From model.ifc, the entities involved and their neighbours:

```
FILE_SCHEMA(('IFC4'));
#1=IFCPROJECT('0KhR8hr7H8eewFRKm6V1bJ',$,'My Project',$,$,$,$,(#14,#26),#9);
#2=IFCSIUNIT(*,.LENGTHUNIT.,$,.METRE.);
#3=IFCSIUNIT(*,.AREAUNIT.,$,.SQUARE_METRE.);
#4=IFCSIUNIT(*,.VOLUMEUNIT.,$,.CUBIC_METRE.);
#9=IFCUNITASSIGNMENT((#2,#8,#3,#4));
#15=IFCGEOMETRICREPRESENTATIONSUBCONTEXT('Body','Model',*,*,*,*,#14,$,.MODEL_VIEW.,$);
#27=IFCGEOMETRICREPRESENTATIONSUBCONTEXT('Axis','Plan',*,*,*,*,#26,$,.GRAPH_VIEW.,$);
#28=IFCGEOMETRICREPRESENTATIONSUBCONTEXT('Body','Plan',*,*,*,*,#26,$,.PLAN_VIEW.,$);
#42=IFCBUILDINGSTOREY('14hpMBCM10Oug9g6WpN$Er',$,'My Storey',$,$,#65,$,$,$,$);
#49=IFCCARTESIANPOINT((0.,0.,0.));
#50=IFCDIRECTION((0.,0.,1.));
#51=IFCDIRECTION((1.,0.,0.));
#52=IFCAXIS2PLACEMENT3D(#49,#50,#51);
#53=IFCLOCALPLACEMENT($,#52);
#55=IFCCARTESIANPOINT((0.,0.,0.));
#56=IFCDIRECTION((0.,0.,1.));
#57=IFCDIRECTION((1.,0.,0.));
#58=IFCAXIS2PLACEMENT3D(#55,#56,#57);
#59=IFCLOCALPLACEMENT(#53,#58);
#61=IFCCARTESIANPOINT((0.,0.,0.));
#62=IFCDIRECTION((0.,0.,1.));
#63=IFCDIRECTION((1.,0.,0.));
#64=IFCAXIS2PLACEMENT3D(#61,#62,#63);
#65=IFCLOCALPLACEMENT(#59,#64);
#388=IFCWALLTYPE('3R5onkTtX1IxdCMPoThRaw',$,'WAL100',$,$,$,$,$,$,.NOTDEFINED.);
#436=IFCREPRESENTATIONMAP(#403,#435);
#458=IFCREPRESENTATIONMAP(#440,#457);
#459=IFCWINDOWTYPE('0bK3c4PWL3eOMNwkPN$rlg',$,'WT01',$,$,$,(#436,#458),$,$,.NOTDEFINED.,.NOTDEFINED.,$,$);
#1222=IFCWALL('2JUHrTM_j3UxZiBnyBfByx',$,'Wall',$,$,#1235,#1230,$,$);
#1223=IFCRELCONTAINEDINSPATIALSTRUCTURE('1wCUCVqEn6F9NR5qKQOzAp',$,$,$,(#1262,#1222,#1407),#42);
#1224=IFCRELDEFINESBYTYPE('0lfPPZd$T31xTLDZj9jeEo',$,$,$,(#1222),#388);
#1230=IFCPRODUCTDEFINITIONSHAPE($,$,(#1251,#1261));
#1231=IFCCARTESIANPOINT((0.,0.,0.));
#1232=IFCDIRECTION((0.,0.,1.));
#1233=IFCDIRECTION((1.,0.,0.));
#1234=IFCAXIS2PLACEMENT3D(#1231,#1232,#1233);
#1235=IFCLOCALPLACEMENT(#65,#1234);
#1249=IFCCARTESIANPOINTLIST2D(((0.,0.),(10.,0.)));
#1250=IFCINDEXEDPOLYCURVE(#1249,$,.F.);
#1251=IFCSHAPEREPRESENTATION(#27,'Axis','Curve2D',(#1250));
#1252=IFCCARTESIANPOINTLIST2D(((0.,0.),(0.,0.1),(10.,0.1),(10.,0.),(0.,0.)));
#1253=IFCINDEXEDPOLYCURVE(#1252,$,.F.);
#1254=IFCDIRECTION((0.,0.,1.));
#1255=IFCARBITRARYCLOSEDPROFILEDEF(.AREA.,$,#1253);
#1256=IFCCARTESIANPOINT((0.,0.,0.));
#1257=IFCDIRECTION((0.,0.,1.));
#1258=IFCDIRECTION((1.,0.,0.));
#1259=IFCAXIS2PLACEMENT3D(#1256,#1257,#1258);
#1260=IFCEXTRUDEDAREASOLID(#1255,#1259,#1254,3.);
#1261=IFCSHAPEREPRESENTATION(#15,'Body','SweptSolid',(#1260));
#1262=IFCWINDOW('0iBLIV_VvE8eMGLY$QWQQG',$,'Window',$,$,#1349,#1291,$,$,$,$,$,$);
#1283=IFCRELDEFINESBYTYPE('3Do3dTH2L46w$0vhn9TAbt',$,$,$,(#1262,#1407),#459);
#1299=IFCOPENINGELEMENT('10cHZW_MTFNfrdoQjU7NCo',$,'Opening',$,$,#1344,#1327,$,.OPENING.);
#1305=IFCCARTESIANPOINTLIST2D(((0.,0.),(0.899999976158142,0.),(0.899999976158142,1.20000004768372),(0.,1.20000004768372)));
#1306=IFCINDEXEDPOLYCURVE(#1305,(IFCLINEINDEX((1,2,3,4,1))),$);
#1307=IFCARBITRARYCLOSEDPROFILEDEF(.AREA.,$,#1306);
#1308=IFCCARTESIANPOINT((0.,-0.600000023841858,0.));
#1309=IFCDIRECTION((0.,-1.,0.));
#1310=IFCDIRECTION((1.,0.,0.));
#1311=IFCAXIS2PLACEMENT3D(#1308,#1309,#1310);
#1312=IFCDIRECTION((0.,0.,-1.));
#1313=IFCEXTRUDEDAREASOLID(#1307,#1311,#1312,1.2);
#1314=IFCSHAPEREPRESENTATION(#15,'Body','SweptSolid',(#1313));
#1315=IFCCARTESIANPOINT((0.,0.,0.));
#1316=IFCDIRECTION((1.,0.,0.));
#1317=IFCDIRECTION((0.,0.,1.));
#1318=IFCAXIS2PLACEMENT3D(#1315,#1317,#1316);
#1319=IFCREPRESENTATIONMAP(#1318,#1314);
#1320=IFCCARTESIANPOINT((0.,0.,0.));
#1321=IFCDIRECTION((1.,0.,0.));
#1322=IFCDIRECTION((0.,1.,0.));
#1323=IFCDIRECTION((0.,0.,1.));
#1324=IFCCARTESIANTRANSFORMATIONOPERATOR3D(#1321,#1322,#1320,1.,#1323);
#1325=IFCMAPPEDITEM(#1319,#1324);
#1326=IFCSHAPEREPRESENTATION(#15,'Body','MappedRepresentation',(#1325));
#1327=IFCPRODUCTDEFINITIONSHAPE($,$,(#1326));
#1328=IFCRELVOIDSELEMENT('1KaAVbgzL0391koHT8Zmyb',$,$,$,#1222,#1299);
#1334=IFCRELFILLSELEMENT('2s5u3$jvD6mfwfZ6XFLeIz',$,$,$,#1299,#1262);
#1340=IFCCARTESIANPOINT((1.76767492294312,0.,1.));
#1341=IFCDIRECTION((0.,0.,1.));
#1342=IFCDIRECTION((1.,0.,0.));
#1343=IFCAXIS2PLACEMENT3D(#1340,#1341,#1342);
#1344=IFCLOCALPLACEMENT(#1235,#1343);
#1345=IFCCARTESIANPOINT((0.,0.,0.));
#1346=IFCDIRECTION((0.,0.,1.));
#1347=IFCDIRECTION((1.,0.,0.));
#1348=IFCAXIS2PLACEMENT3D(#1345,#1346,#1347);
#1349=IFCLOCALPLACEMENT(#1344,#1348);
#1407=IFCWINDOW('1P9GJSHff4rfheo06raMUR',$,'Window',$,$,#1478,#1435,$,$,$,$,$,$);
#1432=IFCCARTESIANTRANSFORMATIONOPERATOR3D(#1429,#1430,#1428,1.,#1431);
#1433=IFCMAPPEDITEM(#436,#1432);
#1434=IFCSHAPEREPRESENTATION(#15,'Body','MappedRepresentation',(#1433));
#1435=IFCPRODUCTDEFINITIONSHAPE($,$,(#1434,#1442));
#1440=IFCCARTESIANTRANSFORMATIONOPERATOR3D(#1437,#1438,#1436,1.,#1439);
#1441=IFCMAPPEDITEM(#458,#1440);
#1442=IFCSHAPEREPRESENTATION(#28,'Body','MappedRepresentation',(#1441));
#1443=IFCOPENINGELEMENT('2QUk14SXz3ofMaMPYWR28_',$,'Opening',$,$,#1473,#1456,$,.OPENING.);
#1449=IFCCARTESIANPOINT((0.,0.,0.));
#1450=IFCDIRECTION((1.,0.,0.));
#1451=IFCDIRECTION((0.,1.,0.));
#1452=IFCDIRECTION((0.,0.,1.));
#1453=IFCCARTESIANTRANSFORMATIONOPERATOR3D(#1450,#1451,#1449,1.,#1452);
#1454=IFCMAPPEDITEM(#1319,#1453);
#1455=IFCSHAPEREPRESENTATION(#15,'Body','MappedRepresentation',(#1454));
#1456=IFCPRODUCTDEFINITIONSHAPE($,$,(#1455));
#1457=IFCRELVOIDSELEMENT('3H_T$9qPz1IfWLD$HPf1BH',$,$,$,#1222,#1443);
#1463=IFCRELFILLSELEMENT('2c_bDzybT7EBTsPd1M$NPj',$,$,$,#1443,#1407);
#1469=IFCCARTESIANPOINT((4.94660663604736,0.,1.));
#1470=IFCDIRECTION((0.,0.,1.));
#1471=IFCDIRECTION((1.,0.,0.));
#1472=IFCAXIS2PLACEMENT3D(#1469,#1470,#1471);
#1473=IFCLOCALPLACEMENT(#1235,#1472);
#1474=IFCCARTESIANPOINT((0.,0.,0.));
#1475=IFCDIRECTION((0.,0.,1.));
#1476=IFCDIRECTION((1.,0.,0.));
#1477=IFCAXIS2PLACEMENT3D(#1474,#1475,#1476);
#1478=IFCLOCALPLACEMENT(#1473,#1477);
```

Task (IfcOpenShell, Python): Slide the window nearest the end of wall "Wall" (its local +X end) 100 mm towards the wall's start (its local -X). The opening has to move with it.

```python
import ifcopenshell
import ifcopenshell.api.geometry
import ifcopenshell.util.placement

model = ifcopenshell.open("model.ifc")

window = model.by_id(1407)
opening = window.FillsVoids[0].RelatingOpeningElement
wall = opening.VoidsElements[0].RelatingBuildingElement

wall_matrix = ifcopenshell.util.placement.get_local_placement(wall.ObjectPlacement)
shift = wall_matrix[:3, 0] * -0.1
before = ifcopenshell.util.placement.get_local_placement(window.ObjectPlacement)[:3, 3].copy()

# The window is placed relative to its opening, so it follows when the opening moves.
matrix = ifcopenshell.util.placement.get_local_placement(opening.ObjectPlacement)
matrix[:3, 3] += shift
ifcopenshell.api.geometry.edit_object_placement(
    model, product=opening, matrix=matrix, is_si=False, should_transform_children=True
)

after = ifcopenshell.util.placement.get_local_placement(window.ObjectPlacement)[:3, 3]
print("window moved by", (after - before).round(3) + 0.0)

model.write("model_v2.ifc")
```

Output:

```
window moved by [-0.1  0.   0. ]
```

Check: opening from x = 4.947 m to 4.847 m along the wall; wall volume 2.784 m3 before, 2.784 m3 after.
